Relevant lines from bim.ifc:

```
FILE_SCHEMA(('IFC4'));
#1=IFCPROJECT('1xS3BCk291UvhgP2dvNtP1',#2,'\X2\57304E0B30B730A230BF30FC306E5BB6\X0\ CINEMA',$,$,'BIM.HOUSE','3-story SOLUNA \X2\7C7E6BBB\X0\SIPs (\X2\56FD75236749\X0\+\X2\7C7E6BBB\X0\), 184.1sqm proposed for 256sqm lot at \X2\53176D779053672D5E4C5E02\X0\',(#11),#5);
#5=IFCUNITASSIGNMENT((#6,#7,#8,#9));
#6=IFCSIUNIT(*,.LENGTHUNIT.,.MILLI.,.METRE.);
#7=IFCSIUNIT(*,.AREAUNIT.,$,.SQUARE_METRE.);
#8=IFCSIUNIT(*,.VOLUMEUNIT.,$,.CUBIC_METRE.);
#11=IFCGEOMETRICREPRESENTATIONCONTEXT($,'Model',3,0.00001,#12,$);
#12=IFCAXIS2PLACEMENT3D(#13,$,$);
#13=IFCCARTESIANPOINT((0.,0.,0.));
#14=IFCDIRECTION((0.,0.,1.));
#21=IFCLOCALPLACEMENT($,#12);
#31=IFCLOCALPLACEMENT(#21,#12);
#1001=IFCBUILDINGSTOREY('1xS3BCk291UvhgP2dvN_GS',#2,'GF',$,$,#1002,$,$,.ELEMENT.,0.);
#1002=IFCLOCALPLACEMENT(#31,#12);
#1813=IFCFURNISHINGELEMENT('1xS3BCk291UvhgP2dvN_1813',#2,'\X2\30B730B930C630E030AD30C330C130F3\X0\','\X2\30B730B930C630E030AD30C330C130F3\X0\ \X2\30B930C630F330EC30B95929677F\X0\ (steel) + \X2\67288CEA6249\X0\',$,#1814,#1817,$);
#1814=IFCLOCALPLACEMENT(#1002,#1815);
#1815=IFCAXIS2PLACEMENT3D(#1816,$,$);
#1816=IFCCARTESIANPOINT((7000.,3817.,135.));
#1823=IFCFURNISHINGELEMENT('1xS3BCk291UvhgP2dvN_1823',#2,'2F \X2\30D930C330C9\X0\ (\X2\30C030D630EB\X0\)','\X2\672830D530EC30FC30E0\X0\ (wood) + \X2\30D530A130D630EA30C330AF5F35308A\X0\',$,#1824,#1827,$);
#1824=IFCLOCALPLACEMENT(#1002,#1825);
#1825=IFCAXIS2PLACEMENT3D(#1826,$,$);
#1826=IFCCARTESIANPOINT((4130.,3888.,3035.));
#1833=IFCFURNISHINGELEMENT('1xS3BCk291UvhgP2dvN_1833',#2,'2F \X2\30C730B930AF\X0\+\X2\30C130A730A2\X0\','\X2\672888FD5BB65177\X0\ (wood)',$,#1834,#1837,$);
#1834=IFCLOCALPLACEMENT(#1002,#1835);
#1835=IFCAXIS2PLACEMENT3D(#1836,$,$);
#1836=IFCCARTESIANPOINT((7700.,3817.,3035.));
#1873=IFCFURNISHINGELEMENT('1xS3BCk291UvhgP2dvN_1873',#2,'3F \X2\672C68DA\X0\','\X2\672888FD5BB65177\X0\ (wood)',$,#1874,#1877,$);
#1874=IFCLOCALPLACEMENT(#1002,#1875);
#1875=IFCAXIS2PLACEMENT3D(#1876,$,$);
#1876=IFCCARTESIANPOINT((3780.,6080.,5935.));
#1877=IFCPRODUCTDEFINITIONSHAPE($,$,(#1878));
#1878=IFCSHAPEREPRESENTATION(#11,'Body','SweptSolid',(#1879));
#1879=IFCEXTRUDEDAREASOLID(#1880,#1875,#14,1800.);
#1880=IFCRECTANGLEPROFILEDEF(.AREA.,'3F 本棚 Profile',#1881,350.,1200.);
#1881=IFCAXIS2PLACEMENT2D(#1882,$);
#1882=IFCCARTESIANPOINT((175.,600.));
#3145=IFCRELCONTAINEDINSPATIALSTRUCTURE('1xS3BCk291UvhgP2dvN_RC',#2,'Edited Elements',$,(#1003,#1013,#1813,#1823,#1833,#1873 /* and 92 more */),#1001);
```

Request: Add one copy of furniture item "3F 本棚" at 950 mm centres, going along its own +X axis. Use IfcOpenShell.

```python
import ifcopenshell
import ifcopenshell.api.geometry
import ifcopenshell.api.root
import ifcopenshell.util.element
import ifcopenshell.util.placement

model = ifcopenshell.open("bim.ifc")


def reuse_history(source, copy):
    """copy_class also copies each property set's owner history, people and application; keep the originals."""
    for rel in copy.IsDefinedBy:
        if rel.is_a("IfcRelDefinesByProperties") and (history := rel.RelatingPropertyDefinition.OwnerHistory):
            rel.RelatingPropertyDefinition.OwnerHistory = source.OwnerHistory
            ifcopenshell.util.element.remove_deep2(model, history)


source = model.by_id(1873)
base = ifcopenshell.util.placement.get_local_placement(source.ObjectPlacement)
step = base[:3, 0] * 950.0

for i in range(1, 2):
    copy = ifcopenshell.api.root.copy_class(model, product=source)
    copy.Representation = ifcopenshell.util.element.copy_deep(
        model, source.Representation, exclude=["IfcGeometricRepresentationContext", "IfcRepresentationMap"]
    )
    reuse_history(source, copy)
    matrix = base.copy()
    matrix[:3, 3] += i * step
    print("added at", matrix[:3, 3].round(3) + 0.0)
    ifcopenshell.api.geometry.edit_object_placement(model, product=copy, matrix=matrix, is_si=False)

model.write("bim_updated.ifc")
```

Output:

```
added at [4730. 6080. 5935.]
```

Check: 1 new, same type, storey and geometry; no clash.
